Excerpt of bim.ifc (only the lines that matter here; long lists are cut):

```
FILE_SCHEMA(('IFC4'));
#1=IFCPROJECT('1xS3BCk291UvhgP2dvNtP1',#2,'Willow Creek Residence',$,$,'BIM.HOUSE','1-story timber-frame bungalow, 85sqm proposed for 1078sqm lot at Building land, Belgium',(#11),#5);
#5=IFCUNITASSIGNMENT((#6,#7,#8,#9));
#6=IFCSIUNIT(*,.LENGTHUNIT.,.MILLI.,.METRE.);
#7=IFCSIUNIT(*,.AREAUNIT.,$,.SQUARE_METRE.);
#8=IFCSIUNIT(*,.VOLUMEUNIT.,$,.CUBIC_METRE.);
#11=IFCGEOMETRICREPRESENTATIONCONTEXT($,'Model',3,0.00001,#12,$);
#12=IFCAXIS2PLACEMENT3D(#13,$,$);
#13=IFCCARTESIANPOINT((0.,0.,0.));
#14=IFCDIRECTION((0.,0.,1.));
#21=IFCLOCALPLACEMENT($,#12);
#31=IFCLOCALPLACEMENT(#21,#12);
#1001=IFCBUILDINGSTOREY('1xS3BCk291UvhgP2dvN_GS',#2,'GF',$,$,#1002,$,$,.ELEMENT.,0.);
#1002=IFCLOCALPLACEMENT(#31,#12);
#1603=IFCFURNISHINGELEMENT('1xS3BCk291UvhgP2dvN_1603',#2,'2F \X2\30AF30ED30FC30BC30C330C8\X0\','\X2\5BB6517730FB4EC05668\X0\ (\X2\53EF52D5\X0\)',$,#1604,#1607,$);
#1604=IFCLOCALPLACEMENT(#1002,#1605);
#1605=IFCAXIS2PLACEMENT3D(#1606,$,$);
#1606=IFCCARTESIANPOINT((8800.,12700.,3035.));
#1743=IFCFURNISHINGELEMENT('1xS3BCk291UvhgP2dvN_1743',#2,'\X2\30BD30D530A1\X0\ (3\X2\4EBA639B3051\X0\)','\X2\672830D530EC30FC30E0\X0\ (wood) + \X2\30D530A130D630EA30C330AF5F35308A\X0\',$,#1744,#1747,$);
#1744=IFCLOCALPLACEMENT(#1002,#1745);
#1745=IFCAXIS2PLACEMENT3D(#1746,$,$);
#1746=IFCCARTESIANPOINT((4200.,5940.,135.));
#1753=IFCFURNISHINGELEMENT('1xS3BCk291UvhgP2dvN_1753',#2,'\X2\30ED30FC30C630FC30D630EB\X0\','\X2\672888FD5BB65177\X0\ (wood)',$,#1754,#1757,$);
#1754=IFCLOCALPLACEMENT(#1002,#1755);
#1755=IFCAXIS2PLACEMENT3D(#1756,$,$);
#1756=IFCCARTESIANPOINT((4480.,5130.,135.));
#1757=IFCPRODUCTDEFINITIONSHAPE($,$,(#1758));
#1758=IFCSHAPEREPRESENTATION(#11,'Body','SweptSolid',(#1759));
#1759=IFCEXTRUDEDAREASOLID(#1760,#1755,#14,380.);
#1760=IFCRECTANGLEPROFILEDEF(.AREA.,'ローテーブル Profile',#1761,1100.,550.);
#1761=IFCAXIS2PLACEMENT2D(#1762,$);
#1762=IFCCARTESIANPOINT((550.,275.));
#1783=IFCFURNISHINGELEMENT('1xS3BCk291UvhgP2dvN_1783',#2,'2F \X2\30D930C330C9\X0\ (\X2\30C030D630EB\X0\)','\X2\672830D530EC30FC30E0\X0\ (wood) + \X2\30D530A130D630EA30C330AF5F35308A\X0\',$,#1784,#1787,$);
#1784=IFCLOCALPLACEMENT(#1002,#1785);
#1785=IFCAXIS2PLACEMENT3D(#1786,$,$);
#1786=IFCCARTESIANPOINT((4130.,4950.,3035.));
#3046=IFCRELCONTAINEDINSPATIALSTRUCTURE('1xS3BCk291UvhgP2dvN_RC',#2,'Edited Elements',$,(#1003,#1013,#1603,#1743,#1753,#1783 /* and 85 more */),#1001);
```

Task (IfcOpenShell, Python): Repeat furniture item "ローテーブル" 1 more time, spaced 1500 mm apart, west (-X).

```python
import numpy as np
import ifcopenshell
import ifcopenshell.api.geometry
import ifcopenshell.api.root
import ifcopenshell.util.element
import ifcopenshell.util.placement

model = ifcopenshell.open("bim.ifc")


def reuse_history(source, copy):
    """copy_class also copies each property set's owner history, people and application; keep the originals."""
    for rel in copy.IsDefinedBy:
        if rel.is_a("IfcRelDefinesByProperties") and (history := rel.RelatingPropertyDefinition.OwnerHistory):
            rel.RelatingPropertyDefinition.OwnerHistory = source.OwnerHistory
            ifcopenshell.util.element.remove_deep2(model, history)


source = model.by_guid("1xS3BCk291UvhgP2dvN_1753")
base = ifcopenshell.util.placement.get_local_placement(source.ObjectPlacement)
step = np.array([-1.0, 0.0, 0.0]) * 1500.0

for i in range(1, 2):
    copy = ifcopenshell.api.root.copy_class(model, product=source)
    copy.Representation = ifcopenshell.util.element.copy_deep(
        model, source.Representation, exclude=["IfcGeometricRepresentationContext", "IfcRepresentationMap"]
    )
    reuse_history(source, copy)
    matrix = base.copy()
    matrix[:3, 3] += i * step
    print("added at", matrix[:3, 3].round(3) + 0.0)
    ifcopenshell.api.geometry.edit_object_placement(model, product=copy, matrix=matrix, is_si=False)

model.write("bim_updated.ifc")
```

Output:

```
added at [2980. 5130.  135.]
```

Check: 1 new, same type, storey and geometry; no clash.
